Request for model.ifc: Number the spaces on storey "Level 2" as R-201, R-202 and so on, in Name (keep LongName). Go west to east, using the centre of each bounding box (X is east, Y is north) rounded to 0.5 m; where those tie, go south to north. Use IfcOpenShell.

First a look at what the model holds.

```python
import ifcopenshell
import ifcopenshell.util.element
import ifcopenshell.util.placement

model = ifcopenshell.open("model.ifc")
print(model.schema)
storey = next(s for s in model.by_type("IfcBuildingStorey") if s.Name == "Level 2")
spaces = [e for e in ifcopenshell.util.element.get_decomposition(storey) if e.is_a("IfcSpace")]
for e in sorted(spaces, key=lambda e: e.id()):
    origin = ifcopenshell.util.placement.get_local_placement(e.ObjectPlacement)[:3, 3]
    print(e.id(), e.Name, e.LongName, origin.round(2) + 0.0, sep=" | ")
```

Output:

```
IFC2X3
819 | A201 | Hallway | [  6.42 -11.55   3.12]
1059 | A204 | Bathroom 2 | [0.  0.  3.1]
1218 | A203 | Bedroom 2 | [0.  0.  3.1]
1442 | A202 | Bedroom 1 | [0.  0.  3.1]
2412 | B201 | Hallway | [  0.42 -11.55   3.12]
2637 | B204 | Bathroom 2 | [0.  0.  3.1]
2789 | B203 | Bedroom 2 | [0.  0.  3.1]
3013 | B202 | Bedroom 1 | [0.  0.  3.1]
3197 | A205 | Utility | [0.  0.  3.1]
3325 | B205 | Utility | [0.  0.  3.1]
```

```python
import ifcopenshell
import ifcopenshell.geom
import ifcopenshell.util.element
import ifcopenshell.util.shape

model = ifcopenshell.open("model.ifc")
settings = ifcopenshell.geom.settings()
settings.set("use-world-coords", True)


def centre(element):
    shape = ifcopenshell.geom.create_shape(settings, element)
    return ifcopenshell.util.shape.get_bbox_centroid(shape.geometry)


storey = next(s for s in model.by_type("IfcBuildingStorey") if s.Name == "Level 2")
spaces = [e for e in ifcopenshell.util.element.get_decomposition(storey) if e.is_a("IfcSpace")]

# Insertion points can sit at a corner or the storey origin, so sort by the geometry (in metres).
centres = {e: centre(e) for e in spaces}
spaces.sort(key=lambda e: (round(centres[e][0] / 0.5), centres[e][1]))

for i, e in enumerate(spaces, start=1):
    number = f"R-2{i:02d}"
    e.Name = number
    print(e.id(), number)

model.write("model-out.ifc")
```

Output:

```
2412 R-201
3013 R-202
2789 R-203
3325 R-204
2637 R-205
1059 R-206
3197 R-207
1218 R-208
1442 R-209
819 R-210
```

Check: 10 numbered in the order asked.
